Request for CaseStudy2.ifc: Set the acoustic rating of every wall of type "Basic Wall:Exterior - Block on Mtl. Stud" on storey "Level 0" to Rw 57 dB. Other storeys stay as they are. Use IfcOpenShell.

First a look at what the model holds.

```python
import ifcopenshell
import ifcopenshell.util.element

model = ifcopenshell.open("CaseStudy2.ifc")
print(model.schema)
storey = next(s for s in model.by_type("IfcBuildingStorey") if s.Name == "Level 0")
walls = [e for e in ifcopenshell.util.element.get_decomposition(storey) if e.is_a("IfcWall")]
seen = {}
for e in walls:
    element_type = ifcopenshell.util.element.get_type(e)
    key = (element_type.Name if element_type != e and element_type else None, ifcopenshell.util.element.get_pset(e, "Pset_WallCommon", "AcousticRating"))
    seen[key] = seen.get(key, 0) + 1
for (name, value), count in sorted(seen.items(), key=str):
    print(count, "x", name, "|", value)
```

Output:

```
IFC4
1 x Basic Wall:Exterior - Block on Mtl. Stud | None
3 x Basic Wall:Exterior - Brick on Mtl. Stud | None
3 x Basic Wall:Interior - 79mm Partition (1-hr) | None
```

```python
import ifcopenshell
import ifcopenshell.api.pset
import ifcopenshell.util.element

model = ifcopenshell.open("CaseStudy2.ifc")

storey = next(s for s in model.by_type("IfcBuildingStorey") if s.Name == "Level 0")
walls = [e for e in ifcopenshell.util.element.get_decomposition(storey) if e.is_a("IfcWall")]

count = 0
for e in walls:
    element_type = ifcopenshell.util.element.get_type(e)
    if element_type in (None, e) or element_type.Name != "Basic Wall:Exterior - Block on Mtl. Stud":
        continue
    # add_pset returns the element's existing set when there is one.
    pset = ifcopenshell.api.pset.add_pset(model, product=e, name="Pset_WallCommon")
    ifcopenshell.api.pset.edit_pset(model, pset=pset, properties={"AcousticRating": "Rw 57 dB"})
    count += 1

print(count, "walls updated")

model.write("CaseStudy2_edited.ifc")
```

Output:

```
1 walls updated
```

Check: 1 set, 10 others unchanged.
